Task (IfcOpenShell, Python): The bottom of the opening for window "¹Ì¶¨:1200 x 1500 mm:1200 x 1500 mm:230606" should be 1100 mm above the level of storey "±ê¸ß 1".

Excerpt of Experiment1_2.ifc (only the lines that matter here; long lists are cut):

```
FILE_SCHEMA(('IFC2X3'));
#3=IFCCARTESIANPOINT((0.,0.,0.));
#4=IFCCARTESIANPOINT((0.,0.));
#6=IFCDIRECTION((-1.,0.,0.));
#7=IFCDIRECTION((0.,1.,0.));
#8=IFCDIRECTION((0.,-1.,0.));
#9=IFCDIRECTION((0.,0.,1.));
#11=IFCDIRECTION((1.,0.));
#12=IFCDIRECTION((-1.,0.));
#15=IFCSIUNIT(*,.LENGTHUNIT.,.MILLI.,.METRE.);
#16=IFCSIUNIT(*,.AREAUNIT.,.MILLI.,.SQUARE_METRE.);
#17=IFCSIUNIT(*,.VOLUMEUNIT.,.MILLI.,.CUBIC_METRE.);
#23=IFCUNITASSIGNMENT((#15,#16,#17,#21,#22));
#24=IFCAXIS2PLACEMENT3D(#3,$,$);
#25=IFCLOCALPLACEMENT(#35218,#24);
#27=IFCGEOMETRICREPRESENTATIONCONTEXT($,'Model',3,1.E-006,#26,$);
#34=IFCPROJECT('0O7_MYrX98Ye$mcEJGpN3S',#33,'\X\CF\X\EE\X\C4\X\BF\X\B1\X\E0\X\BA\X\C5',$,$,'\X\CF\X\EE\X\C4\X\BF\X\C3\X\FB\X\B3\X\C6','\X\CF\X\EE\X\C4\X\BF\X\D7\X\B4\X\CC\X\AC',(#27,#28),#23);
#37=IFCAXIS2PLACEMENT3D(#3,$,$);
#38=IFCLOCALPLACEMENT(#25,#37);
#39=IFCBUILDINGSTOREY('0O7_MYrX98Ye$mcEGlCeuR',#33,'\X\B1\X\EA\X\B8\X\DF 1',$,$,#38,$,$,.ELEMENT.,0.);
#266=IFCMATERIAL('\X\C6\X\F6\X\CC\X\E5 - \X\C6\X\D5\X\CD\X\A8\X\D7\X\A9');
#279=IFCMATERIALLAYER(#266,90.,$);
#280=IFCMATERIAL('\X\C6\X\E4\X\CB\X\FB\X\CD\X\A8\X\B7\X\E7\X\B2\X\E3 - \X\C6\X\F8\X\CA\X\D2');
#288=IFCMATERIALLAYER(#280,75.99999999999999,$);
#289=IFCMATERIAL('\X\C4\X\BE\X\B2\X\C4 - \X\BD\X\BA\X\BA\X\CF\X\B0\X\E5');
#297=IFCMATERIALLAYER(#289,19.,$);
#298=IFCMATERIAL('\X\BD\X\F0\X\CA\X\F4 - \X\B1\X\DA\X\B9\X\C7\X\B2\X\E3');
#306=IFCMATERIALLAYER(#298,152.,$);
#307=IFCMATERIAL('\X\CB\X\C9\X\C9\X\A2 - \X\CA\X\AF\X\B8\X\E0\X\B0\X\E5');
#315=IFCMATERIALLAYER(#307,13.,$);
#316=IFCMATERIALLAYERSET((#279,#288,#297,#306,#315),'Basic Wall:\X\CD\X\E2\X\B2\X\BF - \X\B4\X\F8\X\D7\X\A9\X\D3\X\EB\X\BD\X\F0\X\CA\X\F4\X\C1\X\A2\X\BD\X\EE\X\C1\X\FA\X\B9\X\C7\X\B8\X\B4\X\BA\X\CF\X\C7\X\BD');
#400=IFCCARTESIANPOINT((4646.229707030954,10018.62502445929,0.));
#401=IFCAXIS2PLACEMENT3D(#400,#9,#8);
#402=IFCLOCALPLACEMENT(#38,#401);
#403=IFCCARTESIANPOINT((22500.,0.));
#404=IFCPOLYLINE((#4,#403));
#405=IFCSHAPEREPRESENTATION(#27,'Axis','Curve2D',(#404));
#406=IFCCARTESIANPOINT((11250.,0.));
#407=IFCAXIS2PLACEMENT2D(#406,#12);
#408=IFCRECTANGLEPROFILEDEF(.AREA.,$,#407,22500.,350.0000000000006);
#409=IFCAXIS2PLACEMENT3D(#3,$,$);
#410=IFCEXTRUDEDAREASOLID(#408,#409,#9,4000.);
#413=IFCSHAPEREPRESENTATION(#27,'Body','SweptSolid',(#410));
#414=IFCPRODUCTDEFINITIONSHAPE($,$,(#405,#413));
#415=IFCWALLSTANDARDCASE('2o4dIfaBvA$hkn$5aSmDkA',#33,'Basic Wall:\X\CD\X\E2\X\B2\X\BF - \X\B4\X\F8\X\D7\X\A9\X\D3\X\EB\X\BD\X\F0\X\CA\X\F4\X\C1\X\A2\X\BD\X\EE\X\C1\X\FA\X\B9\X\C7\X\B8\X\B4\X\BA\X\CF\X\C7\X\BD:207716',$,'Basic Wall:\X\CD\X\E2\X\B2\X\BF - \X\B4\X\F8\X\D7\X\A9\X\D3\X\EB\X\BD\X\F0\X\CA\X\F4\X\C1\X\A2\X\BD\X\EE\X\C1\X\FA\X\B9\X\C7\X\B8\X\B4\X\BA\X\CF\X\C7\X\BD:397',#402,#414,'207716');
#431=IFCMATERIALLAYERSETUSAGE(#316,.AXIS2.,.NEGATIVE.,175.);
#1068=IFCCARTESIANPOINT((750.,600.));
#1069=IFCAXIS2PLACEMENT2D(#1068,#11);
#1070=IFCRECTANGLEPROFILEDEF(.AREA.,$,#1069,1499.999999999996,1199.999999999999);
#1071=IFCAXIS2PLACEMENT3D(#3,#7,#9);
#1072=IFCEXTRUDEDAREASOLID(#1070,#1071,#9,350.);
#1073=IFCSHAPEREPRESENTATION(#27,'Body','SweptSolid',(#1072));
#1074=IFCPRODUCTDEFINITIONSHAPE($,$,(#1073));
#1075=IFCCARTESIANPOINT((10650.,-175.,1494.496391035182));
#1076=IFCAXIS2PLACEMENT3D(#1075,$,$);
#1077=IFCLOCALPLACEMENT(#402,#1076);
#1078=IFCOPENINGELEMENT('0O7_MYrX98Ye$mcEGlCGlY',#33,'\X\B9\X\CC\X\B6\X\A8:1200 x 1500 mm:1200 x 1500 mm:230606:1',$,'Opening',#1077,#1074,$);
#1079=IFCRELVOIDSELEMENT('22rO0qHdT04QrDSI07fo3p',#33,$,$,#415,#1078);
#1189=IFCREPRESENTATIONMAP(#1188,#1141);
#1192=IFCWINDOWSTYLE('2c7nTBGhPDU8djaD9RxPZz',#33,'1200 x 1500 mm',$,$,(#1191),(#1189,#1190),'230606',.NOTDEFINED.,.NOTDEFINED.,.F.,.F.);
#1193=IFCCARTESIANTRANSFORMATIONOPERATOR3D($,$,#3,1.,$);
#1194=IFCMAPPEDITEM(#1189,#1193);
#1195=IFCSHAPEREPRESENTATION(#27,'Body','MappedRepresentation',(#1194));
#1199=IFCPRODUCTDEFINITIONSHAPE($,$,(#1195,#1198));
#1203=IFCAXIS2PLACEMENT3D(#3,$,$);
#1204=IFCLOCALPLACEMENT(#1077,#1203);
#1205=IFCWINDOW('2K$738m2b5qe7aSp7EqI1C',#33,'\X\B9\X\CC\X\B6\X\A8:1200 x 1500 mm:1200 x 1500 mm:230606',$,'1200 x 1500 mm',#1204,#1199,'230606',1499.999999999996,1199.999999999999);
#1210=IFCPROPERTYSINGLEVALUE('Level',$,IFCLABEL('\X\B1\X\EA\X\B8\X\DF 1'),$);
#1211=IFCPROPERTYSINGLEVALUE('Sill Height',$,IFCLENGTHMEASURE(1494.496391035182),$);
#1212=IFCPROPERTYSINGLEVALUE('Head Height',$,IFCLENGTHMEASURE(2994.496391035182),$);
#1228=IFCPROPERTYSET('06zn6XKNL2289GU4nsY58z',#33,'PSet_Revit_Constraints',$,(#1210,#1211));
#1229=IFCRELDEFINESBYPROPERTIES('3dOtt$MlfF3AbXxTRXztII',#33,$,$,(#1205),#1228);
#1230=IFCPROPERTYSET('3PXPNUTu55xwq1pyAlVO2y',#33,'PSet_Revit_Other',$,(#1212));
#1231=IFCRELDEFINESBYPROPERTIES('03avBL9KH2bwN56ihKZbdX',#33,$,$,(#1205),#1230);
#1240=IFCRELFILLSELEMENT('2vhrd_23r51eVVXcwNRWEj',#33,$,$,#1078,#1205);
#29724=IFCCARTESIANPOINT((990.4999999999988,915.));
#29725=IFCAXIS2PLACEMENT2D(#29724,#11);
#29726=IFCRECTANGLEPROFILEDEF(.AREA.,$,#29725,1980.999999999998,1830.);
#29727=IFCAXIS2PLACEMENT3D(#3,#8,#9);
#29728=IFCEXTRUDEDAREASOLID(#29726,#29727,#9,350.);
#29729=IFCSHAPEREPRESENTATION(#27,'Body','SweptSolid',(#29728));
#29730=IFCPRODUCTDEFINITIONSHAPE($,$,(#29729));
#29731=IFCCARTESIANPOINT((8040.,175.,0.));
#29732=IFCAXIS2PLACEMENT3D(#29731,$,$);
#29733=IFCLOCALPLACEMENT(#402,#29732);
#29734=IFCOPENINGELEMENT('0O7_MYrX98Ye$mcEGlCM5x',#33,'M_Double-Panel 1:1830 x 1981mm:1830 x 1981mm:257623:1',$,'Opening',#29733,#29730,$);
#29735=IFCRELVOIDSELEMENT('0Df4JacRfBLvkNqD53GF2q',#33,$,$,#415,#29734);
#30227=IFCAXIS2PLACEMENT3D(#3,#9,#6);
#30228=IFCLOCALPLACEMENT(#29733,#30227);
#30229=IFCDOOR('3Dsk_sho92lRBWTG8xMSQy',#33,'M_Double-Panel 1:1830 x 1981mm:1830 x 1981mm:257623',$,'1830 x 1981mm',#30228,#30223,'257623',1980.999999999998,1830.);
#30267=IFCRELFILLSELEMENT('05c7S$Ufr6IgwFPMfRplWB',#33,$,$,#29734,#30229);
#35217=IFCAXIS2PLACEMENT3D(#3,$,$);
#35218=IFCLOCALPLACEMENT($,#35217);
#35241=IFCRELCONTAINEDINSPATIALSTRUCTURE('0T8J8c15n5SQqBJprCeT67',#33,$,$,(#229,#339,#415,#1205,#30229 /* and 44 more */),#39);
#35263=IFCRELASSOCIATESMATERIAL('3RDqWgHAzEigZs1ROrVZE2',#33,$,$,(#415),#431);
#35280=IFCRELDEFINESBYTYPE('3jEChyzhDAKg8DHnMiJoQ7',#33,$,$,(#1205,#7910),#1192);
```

```python
import numpy as np
import ifcopenshell
import ifcopenshell.api.geometry
import ifcopenshell.api.pset
import ifcopenshell.geom
import ifcopenshell.util.element
import ifcopenshell.util.placement
import ifcopenshell.util.shape
import ifcopenshell.util.unit

model = ifcopenshell.open("Experiment1_2.ifc")
unit_scale = ifcopenshell.util.unit.calculate_unit_scale(model)

window = model.by_guid("2K$738m2b5qe7aSp7EqI1C")
opening = window.FillsVoids[0].RelatingOpeningElement
storey = ifcopenshell.util.element.get_container(window, ifc_class="IfcBuildingStorey")
level = ifcopenshell.util.placement.get_local_placement(storey.ObjectPlacement)[2, 3]

# The opening's origin need not be at the sill, so measure its lowest point.
shape = ifcopenshell.geom.create_shape(ifcopenshell.geom.settings(), opening)
bottom = ifcopenshell.util.shape.get_shape_bottom_elevation(shape, shape.geometry) / unit_scale
dz = level + 1.1 / unit_scale - bottom

shift = np.array([0.0, 0.0, dz])
# The window is placed relative to its opening, so it follows when the opening moves.
matrix = ifcopenshell.util.placement.get_local_placement(opening.ObjectPlacement)
matrix[:3, 3] += shift
ifcopenshell.api.geometry.edit_object_placement(
    model, product=opening, matrix=matrix, is_si=False, should_transform_children=True
)

# Keep the stored heights in step.
pset = model.by_id(ifcopenshell.util.element.get_pset(window, "PSet_Revit_Constraints", should_inherit=False)["id"])
ifcopenshell.api.pset.edit_pset(model, pset=pset, properties={
    "Sill Height": model.create_entity("IfcLengthMeasure", ifcopenshell.util.element.get_pset(window, "PSet_Revit_Constraints", "Sill Height") + dz),
})
pset = model.by_id(ifcopenshell.util.element.get_pset(window, "PSet_Revit_Other", should_inherit=False)["id"])
ifcopenshell.api.pset.edit_pset(model, pset=pset, properties={
    "Head Height": model.create_entity("IfcLengthMeasure", ifcopenshell.util.element.get_pset(window, "PSet_Revit_Other", "Head Height") + dz),
})

print(f"moved by {dz * unit_scale:+.3f} m")

model.write("Experiment1_2_edited.ifc")
```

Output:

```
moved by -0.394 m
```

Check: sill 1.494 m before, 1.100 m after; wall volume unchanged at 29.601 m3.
